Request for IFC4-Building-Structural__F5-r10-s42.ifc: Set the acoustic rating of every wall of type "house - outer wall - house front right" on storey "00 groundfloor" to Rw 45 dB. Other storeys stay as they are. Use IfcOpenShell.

First a look at what the model holds.

```python
import ifcopenshell
import ifcopenshell.util.element

model = ifcopenshell.open("IFC4-Building-Structural__F5-r10-s42.ifc")
print(model.schema)
storey = next(s for s in model.by_type("IfcBuildingStorey") if s.Name == "00 groundfloor")
walls = [e for e in ifcopenshell.util.element.get_decomposition(storey) if e.is_a("IfcWall")]
seen = {}
for e in walls:
    element_type = ifcopenshell.util.element.get_type(e)
    key = (element_type.Name if element_type != e and element_type else None, ifcopenshell.util.element.get_pset(e, "Pset_WallCommon", "AcousticRating"))
    seen[key] = seen.get(key, 0) + 1
for (name, value), count in sorted(seen.items(), key=str):
    print(count, "x", name, "|", value)
```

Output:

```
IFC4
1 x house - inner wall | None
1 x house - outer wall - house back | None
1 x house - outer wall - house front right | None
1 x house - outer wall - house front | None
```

```python
import ifcopenshell
import ifcopenshell.api.pset
import ifcopenshell.util.element

model = ifcopenshell.open("IFC4-Building-Structural__F5-r10-s42.ifc")

storey = next(s for s in model.by_type("IfcBuildingStorey") if s.Name == "00 groundfloor")
walls = [e for e in ifcopenshell.util.element.get_decomposition(storey) if e.is_a("IfcWall")]

count = 0
for e in walls:
    element_type = ifcopenshell.util.element.get_type(e)
    if element_type in (None, e) or element_type.Name != "house - outer wall - house front right":
        continue
    # add_pset returns the element's existing set when there is one.
    pset = ifcopenshell.api.pset.add_pset(model, product=e, name="Pset_WallCommon")
    ifcopenshell.api.pset.edit_pset(model, pset=pset, properties={"AcousticRating": "Rw 45 dB"})
    count += 1

print(count, "walls updated")

model.write("IFC4-Building-Structural__F5-r10-s42_v2.ifc")
```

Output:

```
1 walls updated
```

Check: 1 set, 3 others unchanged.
